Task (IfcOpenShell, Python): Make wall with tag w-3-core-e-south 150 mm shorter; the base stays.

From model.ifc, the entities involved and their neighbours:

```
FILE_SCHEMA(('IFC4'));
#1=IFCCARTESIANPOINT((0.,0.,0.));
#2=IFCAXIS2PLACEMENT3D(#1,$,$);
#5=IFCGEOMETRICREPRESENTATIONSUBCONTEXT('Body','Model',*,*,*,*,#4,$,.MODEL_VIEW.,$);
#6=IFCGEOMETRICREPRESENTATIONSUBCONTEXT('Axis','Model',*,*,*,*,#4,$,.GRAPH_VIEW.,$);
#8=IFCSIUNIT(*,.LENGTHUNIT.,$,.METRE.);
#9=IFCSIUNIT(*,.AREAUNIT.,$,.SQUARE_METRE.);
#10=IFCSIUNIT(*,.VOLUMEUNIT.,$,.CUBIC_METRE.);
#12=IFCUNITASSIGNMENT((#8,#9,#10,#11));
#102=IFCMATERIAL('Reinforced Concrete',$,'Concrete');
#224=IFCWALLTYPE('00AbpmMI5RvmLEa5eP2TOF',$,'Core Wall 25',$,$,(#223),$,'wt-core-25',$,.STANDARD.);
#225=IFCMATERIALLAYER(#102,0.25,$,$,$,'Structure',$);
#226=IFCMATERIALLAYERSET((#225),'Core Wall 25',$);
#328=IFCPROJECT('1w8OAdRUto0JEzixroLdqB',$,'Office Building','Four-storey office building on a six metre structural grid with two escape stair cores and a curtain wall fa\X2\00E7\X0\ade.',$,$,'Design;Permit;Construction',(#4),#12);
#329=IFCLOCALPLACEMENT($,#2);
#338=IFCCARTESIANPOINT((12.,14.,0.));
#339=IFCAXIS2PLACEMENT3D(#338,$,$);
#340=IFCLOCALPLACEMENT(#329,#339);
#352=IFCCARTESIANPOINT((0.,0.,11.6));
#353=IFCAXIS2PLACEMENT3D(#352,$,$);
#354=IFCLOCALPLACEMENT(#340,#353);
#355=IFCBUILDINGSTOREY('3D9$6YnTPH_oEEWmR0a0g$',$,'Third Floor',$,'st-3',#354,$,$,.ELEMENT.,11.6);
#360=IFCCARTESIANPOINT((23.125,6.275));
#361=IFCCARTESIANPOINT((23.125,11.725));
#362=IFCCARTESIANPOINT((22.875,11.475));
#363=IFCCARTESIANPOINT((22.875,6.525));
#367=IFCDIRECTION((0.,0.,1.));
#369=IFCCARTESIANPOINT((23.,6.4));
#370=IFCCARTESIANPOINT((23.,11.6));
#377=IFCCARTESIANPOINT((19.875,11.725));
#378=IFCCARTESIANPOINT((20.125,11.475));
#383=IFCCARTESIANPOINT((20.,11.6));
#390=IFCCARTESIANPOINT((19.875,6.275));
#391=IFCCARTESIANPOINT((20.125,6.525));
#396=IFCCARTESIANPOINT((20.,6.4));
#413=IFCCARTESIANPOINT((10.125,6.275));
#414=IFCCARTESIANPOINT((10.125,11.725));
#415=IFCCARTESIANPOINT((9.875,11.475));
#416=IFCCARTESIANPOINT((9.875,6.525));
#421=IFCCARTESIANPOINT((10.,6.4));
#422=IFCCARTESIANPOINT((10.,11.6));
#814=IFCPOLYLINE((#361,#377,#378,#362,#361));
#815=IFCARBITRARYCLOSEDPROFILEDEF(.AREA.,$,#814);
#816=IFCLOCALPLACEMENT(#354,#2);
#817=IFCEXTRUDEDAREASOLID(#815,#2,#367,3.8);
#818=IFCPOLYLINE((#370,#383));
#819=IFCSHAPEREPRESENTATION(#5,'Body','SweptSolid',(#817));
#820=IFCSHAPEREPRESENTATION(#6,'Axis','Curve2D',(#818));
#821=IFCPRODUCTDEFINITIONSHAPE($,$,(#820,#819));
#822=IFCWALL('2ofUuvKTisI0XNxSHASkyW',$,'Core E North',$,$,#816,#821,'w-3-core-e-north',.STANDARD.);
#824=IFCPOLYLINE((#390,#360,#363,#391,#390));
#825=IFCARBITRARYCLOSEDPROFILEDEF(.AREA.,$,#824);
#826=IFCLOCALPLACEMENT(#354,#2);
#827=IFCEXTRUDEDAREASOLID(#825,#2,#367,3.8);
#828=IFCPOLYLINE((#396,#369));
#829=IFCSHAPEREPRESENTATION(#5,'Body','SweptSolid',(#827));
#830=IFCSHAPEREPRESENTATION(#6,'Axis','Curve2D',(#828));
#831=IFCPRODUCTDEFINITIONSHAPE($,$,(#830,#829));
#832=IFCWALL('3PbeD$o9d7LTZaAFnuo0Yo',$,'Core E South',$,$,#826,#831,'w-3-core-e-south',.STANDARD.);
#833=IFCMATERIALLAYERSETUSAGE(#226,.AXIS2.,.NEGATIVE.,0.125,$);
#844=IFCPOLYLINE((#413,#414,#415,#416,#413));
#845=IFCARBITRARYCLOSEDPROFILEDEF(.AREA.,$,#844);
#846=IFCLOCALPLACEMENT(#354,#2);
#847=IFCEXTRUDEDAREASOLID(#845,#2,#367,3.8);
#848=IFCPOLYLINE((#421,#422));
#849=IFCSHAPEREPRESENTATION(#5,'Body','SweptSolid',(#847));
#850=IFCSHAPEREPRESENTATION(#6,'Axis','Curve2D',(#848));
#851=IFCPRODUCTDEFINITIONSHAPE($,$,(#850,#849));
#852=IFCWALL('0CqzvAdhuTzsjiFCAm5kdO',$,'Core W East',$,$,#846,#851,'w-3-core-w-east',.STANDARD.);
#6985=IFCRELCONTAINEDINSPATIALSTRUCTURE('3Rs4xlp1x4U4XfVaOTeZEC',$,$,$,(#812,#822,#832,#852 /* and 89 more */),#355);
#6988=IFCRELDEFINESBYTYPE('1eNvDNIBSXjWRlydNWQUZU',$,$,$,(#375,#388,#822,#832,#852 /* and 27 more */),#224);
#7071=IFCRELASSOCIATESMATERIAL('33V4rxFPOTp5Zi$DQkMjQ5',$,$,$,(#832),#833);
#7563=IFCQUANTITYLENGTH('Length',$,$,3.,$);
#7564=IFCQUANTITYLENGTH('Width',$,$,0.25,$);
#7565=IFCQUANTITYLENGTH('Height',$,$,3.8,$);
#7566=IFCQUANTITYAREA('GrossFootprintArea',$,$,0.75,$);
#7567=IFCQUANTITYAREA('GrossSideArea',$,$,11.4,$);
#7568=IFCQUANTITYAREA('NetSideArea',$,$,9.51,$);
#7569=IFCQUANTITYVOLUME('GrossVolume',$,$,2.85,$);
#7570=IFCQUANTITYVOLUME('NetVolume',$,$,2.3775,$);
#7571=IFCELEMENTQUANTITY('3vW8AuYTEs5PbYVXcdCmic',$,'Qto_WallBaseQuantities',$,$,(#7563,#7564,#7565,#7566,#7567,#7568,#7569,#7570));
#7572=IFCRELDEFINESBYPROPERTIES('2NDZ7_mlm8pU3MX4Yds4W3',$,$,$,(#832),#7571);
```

```python
import ifcopenshell
import ifcopenshell.api.pset
import ifcopenshell.geom
import ifcopenshell.util.element
import ifcopenshell.util.representation
import ifcopenshell.util.shape
import ifcopenshell.util.unit

model = ifcopenshell.open("model.ifc")
unit_scale = ifcopenshell.util.unit.calculate_unit_scale(model)
area_scale = ifcopenshell.util.unit.calculate_unit_scale(model, "AREAUNIT")
volume_scale = ifcopenshell.util.unit.calculate_unit_scale(model, "VOLUMEUNIT")
settings = ifcopenshell.geom.settings()


def volume(element):
    """Net volume in cubic metres, openings subtracted."""
    shape = ifcopenshell.geom.create_shape(settings, element)
    return ifcopenshell.util.shape.get_volume(shape.geometry)


wall = model.by_guid("3PbeD$o9d7LTZaAFnuo0Yo")
before = volume(wall)

body = ifcopenshell.util.representation.get_representation(wall, "Model", "Body")
solid = body.Items[0]
old_height = solid.Depth
solid.Depth -= 0.15
after = volume(wall)
thickness = 0.25  # wall thickness in metres

# Update the stored height, areas and volumes.
qto = model.by_id(ifcopenshell.util.element.get_pset(wall, "Qto_WallBaseQuantities", should_inherit=False)["id"])
ifcopenshell.api.pset.edit_qto(model, qto=qto, properties={
    "Height": solid.Depth,
    "GrossSideArea": ifcopenshell.util.element.get_pset(wall, "Qto_WallBaseQuantities", "GrossSideArea") * solid.Depth / old_height,
    "NetSideArea": after / thickness / area_scale,
    "GrossVolume": ifcopenshell.util.element.get_pset(wall, "Qto_WallBaseQuantities", "GrossVolume") * solid.Depth / old_height,
    "NetVolume": after / volume_scale,
})

print(f"height {old_height:g} -> {solid.Depth:g}, volume {before:.3f} -> {after:.3f} m3")

model.write("model-out.ifc")
```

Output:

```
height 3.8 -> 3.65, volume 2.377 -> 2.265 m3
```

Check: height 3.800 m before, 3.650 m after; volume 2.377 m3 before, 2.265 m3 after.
